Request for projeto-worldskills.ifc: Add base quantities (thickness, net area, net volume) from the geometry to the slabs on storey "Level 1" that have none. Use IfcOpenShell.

First a look at what the model holds.

```python
import ifcopenshell
import ifcopenshell.util.element
import ifcopenshell.util.unit

model = ifcopenshell.open("projeto-worldskills.ifc")
print(model.schema)
for unit_type in ("LENGTHUNIT", "AREAUNIT", "VOLUMEUNIT"):
    print(unit_type, ifcopenshell.util.unit.calculate_unit_scale(model, unit_type))
storey = next(s for s in model.by_type("IfcBuildingStorey") if s.Name == "Level 1")
slabs = [e for e in ifcopenshell.util.element.get_decomposition(storey) if e.is_a("IfcSlab")]
for e in sorted(slabs, key=lambda e: e.id()):
    print(e.id(), e.is_a(), e.Name, list(ifcopenshell.util.element.get_psets(e, qtos_only=True)), sep=" | ")
```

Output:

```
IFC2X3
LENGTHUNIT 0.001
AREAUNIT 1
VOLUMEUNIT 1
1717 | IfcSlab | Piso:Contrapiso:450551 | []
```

```python
import ifcopenshell
import ifcopenshell.api.pset
import ifcopenshell.geom
import ifcopenshell.util.element
import ifcopenshell.util.shape
import ifcopenshell.util.unit

model = ifcopenshell.open("projeto-worldskills.ifc")
unit_scale = ifcopenshell.util.unit.calculate_unit_scale(model)
area_scale = ifcopenshell.util.unit.calculate_unit_scale(model, "AREAUNIT")
volume_scale = ifcopenshell.util.unit.calculate_unit_scale(model, "VOLUMEUNIT")
settings = ifcopenshell.geom.settings()

storey = next(s for s in model.by_type("IfcBuildingStorey") if s.Name == "Level 1")
slabs = [e for e in ifcopenshell.util.element.get_decomposition(storey) if e.is_a("IfcSlab")]

for e in sorted(slabs, key=lambda e: e.id()):
    if ifcopenshell.util.element.get_psets(e, qtos_only=True, should_inherit=False):
        continue
    # Geometry comes back in metres, in the element's own axes.
    shape = ifcopenshell.geom.create_shape(settings, e)
    values = {
        "Width": ifcopenshell.util.shape.get_z(shape.geometry) / unit_scale,
        "NetArea": ifcopenshell.util.shape.get_footprint_area(shape.geometry) / area_scale,
        "NetVolume": ifcopenshell.util.shape.get_volume(shape.geometry) / volume_scale,
    }
    qto = ifcopenshell.api.pset.add_qto(model, product=e, name="BaseQuantities")
    ifcopenshell.api.pset.edit_qto(model, qto=qto, properties=values)
    print(e.id(), {k: round(v, 3) for k, v in values.items()})

model.write("projeto-worldskills_updated.ifc")
```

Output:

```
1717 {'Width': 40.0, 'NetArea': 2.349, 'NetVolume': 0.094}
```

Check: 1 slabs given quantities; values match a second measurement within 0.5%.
